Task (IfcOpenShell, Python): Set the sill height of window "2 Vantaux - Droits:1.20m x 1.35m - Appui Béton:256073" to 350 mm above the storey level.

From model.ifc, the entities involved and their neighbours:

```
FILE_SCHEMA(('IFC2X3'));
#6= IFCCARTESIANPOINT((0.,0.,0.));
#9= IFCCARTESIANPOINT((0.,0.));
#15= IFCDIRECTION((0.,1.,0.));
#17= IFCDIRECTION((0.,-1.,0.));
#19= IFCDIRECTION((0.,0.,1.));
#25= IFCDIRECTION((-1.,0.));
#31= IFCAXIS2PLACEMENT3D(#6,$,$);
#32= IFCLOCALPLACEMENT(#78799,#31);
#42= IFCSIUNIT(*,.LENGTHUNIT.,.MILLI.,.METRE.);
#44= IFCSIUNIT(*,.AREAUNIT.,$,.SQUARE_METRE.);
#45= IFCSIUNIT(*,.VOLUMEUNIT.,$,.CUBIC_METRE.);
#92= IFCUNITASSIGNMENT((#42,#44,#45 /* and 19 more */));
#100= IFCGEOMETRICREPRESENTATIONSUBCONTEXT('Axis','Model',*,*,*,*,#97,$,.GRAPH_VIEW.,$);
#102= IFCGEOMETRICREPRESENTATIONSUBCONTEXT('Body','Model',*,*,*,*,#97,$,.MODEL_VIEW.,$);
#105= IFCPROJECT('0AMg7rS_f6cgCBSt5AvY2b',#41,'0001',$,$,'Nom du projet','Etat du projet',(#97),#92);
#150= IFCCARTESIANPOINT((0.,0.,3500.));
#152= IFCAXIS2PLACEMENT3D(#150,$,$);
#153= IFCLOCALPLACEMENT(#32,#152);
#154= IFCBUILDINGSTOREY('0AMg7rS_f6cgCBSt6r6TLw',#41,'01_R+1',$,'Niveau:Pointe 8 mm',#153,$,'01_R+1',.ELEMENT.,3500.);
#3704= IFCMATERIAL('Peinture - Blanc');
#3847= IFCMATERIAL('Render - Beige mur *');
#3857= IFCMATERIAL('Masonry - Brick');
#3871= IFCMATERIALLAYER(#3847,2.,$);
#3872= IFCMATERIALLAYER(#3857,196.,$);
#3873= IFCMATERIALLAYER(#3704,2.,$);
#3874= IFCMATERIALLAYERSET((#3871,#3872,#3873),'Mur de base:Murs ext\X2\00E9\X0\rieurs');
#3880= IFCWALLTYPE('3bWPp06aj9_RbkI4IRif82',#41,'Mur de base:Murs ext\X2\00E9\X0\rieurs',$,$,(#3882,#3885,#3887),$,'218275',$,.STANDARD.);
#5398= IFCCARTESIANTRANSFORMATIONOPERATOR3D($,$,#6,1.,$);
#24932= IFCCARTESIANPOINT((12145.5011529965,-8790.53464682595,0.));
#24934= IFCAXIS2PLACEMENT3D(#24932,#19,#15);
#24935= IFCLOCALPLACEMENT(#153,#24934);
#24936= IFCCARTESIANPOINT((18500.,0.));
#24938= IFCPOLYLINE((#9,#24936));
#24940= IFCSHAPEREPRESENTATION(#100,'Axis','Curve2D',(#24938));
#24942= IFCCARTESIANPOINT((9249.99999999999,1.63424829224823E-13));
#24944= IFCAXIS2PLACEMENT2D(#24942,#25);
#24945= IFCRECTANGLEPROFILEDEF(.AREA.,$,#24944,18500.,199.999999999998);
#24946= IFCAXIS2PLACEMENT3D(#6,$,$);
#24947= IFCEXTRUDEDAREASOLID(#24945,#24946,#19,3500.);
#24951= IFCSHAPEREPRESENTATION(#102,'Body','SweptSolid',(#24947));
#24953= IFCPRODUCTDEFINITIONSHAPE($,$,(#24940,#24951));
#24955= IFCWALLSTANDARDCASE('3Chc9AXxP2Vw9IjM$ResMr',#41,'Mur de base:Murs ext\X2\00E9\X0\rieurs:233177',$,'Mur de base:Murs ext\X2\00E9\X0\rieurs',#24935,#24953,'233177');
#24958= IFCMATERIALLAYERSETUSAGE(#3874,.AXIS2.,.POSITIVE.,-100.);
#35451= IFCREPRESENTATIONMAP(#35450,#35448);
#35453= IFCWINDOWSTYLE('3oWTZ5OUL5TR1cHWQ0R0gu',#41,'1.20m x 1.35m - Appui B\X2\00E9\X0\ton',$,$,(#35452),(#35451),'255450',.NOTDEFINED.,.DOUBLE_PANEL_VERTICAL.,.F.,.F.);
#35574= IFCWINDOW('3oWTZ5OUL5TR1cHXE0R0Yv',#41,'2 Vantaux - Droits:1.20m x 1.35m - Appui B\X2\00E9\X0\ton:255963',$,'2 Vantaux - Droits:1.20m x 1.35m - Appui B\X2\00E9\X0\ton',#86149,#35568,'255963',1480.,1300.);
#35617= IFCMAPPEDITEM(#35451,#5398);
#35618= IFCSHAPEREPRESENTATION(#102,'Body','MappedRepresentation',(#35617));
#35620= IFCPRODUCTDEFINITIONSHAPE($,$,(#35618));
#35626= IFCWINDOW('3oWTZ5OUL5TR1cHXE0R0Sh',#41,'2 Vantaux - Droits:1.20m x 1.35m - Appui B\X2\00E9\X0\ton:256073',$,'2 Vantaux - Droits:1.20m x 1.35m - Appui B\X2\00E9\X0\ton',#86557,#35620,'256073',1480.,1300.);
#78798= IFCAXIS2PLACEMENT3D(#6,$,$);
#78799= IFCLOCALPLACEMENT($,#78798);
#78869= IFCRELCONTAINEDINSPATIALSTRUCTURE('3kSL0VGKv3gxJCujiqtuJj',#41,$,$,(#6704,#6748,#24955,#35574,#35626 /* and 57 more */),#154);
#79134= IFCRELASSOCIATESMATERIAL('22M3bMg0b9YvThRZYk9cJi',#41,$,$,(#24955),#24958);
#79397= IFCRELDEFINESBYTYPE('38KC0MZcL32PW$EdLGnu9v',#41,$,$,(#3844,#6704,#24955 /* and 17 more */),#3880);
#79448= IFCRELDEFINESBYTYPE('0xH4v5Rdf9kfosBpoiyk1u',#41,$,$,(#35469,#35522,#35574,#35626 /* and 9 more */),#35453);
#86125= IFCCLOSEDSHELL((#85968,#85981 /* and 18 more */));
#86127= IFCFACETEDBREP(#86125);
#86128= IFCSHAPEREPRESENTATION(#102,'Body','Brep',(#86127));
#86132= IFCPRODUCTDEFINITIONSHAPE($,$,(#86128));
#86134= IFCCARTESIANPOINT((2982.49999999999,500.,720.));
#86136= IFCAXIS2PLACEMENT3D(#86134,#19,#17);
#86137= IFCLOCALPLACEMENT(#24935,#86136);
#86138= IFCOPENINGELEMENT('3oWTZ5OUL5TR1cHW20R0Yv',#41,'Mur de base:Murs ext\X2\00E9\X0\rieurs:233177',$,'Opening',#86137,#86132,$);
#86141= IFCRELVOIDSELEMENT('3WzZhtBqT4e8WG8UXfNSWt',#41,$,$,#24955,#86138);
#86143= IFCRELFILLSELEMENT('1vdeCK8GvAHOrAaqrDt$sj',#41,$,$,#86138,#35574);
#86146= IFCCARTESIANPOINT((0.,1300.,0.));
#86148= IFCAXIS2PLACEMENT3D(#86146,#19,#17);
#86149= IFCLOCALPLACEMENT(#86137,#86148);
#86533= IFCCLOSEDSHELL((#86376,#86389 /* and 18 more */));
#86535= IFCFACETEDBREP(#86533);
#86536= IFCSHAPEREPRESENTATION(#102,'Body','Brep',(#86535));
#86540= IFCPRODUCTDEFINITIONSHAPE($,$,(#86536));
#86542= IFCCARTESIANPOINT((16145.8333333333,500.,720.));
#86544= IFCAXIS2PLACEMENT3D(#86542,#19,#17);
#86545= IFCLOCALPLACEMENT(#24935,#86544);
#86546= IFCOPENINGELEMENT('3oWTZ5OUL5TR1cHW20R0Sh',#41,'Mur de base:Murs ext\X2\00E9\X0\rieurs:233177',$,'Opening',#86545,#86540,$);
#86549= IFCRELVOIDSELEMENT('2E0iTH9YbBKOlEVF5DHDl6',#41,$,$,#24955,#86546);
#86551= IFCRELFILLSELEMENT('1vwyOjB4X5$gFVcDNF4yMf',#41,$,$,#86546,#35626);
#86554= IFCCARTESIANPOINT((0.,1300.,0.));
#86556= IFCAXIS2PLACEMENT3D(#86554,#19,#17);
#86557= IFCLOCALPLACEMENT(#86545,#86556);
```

```python
import numpy as np
import ifcopenshell
import ifcopenshell.api.geometry
import ifcopenshell.geom
import ifcopenshell.util.element
import ifcopenshell.util.placement
import ifcopenshell.util.shape
import ifcopenshell.util.unit

model = ifcopenshell.open("model.ifc")
unit_scale = ifcopenshell.util.unit.calculate_unit_scale(model)

window = model.by_id(35626)
opening = window.FillsVoids[0].RelatingOpeningElement
storey = ifcopenshell.util.element.get_container(window, ifc_class="IfcBuildingStorey")
level = ifcopenshell.util.placement.get_local_placement(storey.ObjectPlacement)[2, 3]

# The opening's origin need not be at the sill, so measure its lowest point.
shape = ifcopenshell.geom.create_shape(ifcopenshell.geom.settings(), opening)
bottom = ifcopenshell.util.shape.get_shape_bottom_elevation(shape, shape.geometry) / unit_scale
dz = level + 350.0 - bottom

shift = np.array([0.0, 0.0, dz])
# The window is placed relative to its opening, so it follows when the opening moves.
matrix = ifcopenshell.util.placement.get_local_placement(opening.ObjectPlacement)
matrix[:3, 3] += shift
ifcopenshell.api.geometry.edit_object_placement(
    model, product=opening, matrix=matrix, is_si=False, should_transform_children=True
)

print(f"moved by {dz * unit_scale:+.3f} m")

model.write("model_edited.ifc")
```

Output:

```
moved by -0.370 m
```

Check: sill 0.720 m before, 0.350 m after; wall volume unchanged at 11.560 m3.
